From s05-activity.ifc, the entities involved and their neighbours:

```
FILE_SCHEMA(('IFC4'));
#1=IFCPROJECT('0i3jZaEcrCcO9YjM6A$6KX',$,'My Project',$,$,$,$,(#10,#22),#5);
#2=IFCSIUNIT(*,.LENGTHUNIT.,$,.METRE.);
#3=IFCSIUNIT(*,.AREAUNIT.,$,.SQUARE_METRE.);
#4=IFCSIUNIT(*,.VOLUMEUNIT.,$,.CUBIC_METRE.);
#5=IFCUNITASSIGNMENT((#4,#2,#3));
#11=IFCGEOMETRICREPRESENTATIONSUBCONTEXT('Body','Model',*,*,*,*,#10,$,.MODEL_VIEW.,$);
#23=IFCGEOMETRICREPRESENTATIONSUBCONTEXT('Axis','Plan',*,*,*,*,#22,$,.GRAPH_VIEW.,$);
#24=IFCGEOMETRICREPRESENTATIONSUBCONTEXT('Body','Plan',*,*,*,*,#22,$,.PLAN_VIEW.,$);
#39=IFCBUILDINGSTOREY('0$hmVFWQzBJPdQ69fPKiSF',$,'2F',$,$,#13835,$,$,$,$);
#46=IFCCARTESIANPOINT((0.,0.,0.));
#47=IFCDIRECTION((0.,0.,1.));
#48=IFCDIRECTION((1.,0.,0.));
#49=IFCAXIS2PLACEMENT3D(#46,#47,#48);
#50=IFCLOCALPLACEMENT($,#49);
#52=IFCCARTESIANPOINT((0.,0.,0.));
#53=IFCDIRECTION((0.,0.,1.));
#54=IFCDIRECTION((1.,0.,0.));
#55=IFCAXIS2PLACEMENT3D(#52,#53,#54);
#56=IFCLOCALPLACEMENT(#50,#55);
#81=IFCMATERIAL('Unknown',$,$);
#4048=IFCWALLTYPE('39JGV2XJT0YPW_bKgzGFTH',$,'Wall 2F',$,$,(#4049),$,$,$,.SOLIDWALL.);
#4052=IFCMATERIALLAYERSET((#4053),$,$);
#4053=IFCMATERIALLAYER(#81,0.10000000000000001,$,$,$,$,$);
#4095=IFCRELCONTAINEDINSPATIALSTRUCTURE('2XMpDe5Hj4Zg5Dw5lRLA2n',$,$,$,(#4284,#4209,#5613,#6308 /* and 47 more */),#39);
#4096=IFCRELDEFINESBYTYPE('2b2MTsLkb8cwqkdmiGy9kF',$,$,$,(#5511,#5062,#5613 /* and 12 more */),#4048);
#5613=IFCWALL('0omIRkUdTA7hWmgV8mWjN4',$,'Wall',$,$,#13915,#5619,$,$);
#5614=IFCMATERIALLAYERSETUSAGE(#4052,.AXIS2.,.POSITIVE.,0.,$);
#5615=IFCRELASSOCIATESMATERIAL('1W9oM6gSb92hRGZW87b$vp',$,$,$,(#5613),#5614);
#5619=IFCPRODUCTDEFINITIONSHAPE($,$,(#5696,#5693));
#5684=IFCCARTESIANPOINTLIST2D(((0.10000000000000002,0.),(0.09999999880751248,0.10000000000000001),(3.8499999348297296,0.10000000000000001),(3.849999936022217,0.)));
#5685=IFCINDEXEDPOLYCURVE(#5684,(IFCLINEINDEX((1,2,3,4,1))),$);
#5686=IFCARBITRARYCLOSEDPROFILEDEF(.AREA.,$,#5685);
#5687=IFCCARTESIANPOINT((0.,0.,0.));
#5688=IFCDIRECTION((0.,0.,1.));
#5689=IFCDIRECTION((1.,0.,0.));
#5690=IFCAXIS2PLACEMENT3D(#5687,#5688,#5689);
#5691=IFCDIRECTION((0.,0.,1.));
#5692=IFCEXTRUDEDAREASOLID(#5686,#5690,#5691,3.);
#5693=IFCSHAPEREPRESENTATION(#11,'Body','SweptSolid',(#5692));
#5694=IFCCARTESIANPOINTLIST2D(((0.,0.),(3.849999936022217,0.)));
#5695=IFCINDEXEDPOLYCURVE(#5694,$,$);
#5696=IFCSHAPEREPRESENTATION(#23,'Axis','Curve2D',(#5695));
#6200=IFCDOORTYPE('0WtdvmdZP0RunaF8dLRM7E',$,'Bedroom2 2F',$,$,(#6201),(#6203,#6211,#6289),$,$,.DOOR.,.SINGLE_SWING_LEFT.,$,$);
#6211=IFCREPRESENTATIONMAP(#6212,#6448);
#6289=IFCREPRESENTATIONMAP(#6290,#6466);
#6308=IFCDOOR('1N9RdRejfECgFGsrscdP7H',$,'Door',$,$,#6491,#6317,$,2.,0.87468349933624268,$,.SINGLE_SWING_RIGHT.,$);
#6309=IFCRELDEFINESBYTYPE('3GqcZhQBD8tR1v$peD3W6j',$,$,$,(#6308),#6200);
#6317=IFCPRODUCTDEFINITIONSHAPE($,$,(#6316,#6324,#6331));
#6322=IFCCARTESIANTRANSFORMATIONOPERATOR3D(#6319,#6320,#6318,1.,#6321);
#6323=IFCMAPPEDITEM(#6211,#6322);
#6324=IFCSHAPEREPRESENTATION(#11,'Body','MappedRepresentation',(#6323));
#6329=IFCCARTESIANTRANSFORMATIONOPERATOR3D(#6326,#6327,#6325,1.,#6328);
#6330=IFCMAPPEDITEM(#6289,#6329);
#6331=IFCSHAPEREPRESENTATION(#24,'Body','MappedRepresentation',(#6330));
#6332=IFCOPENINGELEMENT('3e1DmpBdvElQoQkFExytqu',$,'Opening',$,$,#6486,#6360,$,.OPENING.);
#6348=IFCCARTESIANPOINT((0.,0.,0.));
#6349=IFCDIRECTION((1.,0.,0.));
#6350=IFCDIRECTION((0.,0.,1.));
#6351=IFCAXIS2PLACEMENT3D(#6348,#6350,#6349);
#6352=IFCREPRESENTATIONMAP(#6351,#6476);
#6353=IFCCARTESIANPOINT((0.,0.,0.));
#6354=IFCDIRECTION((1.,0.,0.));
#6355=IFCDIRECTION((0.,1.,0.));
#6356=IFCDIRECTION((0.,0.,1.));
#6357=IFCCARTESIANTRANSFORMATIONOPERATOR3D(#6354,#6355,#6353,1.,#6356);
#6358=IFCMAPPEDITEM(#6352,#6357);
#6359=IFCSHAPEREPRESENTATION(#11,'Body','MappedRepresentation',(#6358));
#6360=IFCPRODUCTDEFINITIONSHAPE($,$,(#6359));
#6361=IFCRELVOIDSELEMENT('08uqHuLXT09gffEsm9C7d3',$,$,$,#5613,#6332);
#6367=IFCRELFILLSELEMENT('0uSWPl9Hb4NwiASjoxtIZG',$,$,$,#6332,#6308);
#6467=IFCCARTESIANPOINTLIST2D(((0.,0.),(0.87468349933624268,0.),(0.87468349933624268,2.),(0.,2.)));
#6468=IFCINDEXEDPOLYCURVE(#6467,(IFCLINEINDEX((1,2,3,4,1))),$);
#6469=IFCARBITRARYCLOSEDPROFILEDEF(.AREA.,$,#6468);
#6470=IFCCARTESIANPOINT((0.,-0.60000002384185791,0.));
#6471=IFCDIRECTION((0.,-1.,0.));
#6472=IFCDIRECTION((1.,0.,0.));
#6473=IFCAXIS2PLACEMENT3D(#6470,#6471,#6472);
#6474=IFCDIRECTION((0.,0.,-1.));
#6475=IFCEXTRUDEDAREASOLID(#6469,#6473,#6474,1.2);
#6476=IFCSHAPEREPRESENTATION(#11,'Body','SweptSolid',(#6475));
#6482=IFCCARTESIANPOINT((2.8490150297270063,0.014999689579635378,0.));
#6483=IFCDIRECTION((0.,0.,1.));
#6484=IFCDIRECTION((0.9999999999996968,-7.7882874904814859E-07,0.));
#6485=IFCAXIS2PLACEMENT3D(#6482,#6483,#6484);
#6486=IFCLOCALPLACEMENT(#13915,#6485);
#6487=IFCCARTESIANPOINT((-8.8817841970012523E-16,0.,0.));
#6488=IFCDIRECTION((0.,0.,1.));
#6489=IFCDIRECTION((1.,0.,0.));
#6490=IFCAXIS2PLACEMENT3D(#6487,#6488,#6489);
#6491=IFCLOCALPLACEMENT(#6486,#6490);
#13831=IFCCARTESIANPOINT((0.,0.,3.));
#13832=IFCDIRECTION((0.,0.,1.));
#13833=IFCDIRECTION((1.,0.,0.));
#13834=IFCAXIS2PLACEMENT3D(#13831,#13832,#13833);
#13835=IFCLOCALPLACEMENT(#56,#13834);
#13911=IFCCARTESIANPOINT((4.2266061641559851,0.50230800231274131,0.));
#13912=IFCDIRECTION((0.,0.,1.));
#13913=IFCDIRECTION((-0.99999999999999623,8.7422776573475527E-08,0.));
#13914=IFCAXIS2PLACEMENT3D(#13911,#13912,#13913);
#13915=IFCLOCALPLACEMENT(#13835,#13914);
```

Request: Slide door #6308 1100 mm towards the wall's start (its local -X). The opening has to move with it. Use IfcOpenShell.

```python
import ifcopenshell
import ifcopenshell.api.geometry
import ifcopenshell.util.placement

model = ifcopenshell.open("s05-activity.ifc")

door = model.by_guid("1N9RdRejfECgFGsrscdP7H")
opening = door.FillsVoids[0].RelatingOpeningElement
wall = opening.VoidsElements[0].RelatingBuildingElement

wall_matrix = ifcopenshell.util.placement.get_local_placement(wall.ObjectPlacement)
shift = wall_matrix[:3, 0] * -1.1
before = ifcopenshell.util.placement.get_local_placement(door.ObjectPlacement)[:3, 3].copy()

# The door is placed relative to its opening, so it follows when the opening moves.
matrix = ifcopenshell.util.placement.get_local_placement(opening.ObjectPlacement)
matrix[:3, 3] += shift
ifcopenshell.api.geometry.edit_object_placement(
    model, product=opening, matrix=matrix, is_si=False, should_transform_children=True
)

after = ifcopenshell.util.placement.get_local_placement(door.ObjectPlacement)[:3, 3]
print("door moved by", (after - before).round(3) + 0.0)

model.write("s05-activity_edited.ifc")
```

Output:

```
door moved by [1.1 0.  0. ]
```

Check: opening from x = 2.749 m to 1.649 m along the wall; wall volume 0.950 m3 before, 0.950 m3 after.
